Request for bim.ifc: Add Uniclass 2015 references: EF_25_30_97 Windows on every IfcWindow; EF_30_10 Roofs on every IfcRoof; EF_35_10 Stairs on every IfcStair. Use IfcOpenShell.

First a look at what the model holds.

```python
import ifcopenshell

model = ifcopenshell.open("bim.ifc")
print(model.schema)
print("classifications:", [c.Name for c in model.by_type("IfcClassification")])
for ifc_class in ("IfcDoor", "IfcRoof", "IfcStair", "IfcWall", "IfcWindow"):
    print(ifc_class, len(model.by_type(ifc_class)))
```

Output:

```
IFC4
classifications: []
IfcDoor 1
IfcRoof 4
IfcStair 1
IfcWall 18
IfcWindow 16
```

```python
import ifcopenshell
import ifcopenshell.api.classification

model = ifcopenshell.open("bim.ifc")

system = ifcopenshell.api.classification.add_classification(model, classification="Uniclass 2015")

codes = {
    "IfcWindow": ("EF_25_30_97", "Windows"),
    "IfcRoof": ("EF_30_10", "Roofs"),
    "IfcStair": ("EF_35_10", "Stairs"),
}
for ifc_class, (code, name) in codes.items():
    products = model.by_type(ifc_class)
    ifcopenshell.api.classification.add_reference(
        model, products=products, classification=system, identification=code, name=name
    )
    print(code, len(products))

model.write("bim_edited.ifc")
```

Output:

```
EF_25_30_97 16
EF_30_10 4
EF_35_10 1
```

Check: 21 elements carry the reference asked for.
